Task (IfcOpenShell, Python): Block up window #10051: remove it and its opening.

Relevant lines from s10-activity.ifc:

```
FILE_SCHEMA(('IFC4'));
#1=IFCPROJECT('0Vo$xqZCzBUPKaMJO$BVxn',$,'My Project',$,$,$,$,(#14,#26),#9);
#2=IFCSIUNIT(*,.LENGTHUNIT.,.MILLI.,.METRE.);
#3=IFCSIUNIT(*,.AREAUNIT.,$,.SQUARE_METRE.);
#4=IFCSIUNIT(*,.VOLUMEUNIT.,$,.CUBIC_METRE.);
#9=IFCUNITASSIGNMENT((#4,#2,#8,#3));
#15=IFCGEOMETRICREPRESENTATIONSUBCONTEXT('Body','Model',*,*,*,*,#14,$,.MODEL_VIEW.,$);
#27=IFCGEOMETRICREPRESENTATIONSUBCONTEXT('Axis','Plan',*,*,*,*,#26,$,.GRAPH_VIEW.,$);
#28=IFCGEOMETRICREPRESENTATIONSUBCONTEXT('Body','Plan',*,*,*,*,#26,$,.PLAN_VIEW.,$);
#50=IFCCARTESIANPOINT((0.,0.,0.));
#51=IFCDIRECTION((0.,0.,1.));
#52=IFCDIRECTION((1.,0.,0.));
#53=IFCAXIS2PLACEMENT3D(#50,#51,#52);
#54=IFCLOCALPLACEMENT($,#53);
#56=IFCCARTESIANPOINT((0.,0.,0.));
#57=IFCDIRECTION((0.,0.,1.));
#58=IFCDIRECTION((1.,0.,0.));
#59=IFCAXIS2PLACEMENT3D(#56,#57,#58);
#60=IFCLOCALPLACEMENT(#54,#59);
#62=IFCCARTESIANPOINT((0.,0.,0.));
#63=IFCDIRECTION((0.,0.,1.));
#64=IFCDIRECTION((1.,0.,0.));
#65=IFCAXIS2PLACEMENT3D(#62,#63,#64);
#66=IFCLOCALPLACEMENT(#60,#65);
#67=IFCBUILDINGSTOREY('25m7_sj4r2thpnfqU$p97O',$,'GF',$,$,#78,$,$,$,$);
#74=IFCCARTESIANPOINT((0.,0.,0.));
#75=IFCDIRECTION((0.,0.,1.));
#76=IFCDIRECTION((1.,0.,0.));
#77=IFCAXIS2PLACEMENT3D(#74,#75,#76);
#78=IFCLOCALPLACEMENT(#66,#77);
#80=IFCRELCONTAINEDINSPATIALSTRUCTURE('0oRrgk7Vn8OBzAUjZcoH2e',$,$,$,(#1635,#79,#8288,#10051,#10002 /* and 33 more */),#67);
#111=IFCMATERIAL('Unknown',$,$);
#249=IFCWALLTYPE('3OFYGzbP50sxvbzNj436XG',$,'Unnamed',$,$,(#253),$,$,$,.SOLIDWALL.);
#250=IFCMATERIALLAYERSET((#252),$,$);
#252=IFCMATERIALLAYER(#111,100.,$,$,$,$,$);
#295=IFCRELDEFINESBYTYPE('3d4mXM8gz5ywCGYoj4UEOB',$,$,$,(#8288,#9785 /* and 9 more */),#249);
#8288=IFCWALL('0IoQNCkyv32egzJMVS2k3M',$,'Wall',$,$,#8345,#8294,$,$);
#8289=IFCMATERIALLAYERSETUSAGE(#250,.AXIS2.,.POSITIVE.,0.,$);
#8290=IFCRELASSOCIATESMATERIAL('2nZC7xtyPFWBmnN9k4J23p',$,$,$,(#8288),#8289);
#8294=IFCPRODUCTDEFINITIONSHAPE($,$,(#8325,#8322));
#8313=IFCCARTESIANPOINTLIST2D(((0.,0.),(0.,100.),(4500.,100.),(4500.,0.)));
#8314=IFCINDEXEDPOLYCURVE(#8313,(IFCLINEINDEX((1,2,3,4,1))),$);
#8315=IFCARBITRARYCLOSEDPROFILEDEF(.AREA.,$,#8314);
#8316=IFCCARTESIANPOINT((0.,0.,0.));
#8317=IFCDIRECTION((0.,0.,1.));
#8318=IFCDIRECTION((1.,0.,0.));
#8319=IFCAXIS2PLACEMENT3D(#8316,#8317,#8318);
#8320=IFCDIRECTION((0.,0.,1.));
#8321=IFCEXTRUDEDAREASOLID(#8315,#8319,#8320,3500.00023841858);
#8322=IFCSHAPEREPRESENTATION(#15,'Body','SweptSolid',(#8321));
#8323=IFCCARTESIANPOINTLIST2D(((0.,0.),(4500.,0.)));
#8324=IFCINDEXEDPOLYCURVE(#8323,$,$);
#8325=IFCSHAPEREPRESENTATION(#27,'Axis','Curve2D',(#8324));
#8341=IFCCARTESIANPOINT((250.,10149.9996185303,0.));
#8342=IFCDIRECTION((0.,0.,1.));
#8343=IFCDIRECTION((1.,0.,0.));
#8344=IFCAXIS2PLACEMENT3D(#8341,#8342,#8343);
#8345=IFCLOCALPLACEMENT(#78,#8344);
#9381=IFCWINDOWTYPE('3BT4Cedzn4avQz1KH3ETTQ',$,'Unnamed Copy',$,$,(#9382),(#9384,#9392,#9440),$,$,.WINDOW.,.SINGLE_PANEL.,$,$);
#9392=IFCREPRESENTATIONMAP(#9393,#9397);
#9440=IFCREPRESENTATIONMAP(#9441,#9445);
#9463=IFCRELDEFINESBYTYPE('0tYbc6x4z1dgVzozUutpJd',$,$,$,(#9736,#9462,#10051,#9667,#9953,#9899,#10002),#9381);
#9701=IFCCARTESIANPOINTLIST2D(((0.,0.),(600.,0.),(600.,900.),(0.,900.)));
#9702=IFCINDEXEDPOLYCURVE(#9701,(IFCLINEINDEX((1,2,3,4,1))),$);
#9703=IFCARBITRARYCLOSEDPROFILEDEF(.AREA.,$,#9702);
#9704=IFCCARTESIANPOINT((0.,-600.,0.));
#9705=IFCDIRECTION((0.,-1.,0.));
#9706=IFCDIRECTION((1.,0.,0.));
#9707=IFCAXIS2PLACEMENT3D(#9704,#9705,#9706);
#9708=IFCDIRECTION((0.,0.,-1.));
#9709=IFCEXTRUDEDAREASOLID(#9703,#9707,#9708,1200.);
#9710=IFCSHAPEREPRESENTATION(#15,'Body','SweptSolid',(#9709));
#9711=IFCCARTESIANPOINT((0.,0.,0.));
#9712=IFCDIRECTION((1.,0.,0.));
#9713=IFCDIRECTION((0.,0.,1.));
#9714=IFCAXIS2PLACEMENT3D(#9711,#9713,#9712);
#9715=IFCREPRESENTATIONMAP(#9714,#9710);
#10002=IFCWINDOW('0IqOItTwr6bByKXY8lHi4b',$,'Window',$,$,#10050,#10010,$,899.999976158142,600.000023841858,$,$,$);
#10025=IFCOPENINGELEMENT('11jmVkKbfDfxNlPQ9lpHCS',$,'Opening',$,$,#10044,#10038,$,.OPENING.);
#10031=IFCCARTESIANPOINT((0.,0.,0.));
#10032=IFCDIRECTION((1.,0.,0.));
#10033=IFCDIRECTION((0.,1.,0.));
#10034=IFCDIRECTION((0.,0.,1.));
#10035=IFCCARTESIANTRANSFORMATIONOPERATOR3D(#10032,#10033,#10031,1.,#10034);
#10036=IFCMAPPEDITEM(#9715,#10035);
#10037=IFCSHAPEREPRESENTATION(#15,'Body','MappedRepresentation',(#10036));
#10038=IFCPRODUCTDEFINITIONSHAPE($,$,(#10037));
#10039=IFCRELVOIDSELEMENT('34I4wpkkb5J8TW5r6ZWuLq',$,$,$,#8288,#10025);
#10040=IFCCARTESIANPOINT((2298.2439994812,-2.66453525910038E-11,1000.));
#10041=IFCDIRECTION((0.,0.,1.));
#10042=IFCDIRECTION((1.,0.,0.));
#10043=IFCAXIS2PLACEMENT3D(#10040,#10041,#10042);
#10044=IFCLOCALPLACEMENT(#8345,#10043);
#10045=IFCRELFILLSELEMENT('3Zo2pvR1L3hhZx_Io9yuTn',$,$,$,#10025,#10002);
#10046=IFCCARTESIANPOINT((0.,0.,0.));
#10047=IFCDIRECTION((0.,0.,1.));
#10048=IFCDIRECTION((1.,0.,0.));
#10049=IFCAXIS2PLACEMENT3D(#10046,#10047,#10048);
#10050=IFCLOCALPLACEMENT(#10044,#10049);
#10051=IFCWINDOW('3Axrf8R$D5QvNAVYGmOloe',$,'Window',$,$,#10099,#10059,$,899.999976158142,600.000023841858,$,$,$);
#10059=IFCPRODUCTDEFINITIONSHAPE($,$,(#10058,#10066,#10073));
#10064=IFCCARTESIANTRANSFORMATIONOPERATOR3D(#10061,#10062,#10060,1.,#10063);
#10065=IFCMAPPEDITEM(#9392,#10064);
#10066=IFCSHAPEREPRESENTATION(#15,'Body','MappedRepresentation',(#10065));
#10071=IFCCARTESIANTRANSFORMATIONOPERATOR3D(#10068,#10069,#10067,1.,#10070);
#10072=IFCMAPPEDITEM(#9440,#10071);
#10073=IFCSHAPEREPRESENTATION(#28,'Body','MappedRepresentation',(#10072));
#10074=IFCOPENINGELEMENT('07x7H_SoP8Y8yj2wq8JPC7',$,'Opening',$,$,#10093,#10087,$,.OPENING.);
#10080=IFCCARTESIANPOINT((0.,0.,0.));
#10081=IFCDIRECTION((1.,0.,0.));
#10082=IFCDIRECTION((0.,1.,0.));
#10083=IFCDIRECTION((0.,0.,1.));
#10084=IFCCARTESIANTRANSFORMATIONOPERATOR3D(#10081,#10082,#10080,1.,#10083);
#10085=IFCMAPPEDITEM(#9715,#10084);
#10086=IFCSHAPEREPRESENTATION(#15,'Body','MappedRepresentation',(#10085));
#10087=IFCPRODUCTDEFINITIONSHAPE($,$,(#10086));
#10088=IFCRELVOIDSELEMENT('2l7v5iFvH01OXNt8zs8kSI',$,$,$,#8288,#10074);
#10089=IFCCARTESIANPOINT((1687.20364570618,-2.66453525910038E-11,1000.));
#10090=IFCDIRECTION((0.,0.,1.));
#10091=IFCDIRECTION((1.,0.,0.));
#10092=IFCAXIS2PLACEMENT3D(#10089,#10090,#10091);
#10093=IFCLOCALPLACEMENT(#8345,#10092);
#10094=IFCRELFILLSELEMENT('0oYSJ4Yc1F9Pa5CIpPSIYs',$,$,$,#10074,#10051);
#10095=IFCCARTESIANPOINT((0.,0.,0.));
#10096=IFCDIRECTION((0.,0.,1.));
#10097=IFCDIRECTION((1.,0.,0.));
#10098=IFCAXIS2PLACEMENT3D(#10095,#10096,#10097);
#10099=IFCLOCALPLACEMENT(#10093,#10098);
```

```python
import ifcopenshell
import ifcopenshell.api.feature
import ifcopenshell.api.root
import ifcopenshell.geom
import ifcopenshell.util.shape

model = ifcopenshell.open("s10-activity.ifc")
settings = ifcopenshell.geom.settings()


def volume(element):
    """Net volume in cubic metres, openings subtracted."""
    shape = ifcopenshell.geom.create_shape(settings, element)
    return ifcopenshell.util.shape.get_volume(shape.geometry)


window = model.by_guid("3Axrf8R$D5QvNAVYGmOloe")
opening = window.FillsVoids[0].RelatingOpeningElement
wall = opening.VoidsElements[0].RelatingBuildingElement
before = volume(wall)

ifcopenshell.api.root.remove_product(model, product=window)
ifcopenshell.api.feature.remove_feature(model, feature=opening)

after = volume(wall)

print(f"wall volume {before:.3f} -> {after:.3f} m3")

model.write("s10-activity_edited.ifc")
```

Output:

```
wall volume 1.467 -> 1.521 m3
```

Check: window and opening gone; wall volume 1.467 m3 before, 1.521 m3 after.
